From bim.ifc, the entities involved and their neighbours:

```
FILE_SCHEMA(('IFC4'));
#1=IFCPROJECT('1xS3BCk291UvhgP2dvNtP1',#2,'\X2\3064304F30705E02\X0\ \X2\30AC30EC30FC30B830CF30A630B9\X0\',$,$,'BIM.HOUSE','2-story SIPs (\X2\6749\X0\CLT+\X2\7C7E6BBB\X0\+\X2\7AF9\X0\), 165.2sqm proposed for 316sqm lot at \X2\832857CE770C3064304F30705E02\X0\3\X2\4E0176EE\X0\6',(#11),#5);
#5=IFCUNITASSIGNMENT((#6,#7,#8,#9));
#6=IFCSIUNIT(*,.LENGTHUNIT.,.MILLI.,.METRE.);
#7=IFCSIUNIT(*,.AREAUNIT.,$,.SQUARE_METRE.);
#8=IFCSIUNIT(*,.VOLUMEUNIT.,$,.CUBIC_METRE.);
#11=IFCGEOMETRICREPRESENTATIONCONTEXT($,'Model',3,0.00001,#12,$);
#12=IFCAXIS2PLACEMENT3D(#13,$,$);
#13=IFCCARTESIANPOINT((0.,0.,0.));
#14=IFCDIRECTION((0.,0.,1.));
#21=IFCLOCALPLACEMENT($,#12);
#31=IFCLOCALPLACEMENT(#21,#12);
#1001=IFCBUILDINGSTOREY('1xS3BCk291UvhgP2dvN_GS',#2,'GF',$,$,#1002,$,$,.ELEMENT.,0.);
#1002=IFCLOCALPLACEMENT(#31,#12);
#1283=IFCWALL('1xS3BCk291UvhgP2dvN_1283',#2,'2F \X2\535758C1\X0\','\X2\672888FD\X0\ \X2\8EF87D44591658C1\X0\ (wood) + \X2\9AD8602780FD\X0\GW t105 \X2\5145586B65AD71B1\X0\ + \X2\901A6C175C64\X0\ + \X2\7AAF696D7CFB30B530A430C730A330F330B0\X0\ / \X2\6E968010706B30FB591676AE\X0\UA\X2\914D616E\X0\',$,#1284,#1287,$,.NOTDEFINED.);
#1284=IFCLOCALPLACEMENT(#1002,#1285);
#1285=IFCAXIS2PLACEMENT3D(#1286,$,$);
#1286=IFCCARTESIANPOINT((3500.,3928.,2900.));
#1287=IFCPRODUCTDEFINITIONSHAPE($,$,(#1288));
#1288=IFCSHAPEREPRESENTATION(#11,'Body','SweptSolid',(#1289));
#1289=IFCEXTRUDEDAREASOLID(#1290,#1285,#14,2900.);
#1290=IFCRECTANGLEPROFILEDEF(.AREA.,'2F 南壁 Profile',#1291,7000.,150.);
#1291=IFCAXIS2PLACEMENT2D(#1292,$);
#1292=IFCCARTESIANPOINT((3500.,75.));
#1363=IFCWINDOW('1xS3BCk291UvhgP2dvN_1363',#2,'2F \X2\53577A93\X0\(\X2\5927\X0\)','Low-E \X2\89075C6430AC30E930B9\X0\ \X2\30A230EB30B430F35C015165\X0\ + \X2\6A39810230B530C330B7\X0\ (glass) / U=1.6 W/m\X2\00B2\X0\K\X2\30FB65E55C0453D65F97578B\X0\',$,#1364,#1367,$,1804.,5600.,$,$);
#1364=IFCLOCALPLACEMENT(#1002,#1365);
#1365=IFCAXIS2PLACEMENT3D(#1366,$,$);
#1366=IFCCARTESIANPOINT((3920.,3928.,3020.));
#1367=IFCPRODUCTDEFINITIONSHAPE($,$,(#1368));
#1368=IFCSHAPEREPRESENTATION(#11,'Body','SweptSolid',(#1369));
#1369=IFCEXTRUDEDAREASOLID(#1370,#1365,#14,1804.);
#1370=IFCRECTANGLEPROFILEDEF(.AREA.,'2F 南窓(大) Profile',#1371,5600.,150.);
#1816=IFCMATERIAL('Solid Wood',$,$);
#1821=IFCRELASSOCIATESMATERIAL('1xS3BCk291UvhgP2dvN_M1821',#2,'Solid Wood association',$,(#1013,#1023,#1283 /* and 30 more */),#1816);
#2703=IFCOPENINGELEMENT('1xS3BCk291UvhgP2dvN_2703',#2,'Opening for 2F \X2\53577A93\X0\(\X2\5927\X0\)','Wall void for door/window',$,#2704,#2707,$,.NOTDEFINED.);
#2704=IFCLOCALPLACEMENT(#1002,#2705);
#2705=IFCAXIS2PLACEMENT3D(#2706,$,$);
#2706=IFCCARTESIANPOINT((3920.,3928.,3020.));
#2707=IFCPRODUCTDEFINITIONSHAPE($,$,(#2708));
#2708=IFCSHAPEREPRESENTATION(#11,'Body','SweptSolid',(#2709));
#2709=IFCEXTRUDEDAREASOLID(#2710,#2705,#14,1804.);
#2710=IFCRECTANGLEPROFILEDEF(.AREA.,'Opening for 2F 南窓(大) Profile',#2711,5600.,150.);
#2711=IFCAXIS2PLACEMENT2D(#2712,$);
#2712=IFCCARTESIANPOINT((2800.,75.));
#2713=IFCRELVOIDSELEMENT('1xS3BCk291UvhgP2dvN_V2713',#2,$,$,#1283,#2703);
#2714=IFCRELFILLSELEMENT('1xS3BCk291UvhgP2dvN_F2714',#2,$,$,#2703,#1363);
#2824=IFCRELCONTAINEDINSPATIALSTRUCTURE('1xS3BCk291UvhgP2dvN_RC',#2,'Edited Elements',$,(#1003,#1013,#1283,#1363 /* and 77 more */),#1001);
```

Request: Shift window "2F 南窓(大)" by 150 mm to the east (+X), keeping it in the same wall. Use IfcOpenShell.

```python
import ifcopenshell
import ifcopenshell.api.geometry
import ifcopenshell.util.placement
import ifcopenshell.util.unit

model = ifcopenshell.open("bim.ifc")
unit_scale = ifcopenshell.util.unit.calculate_unit_scale(model)

window = model.by_guid("1xS3BCk291UvhgP2dvN_1363")
opening = window.FillsVoids[0].RelatingOpeningElement
wall = opening.VoidsElements[0].RelatingBuildingElement

wall_matrix = ifcopenshell.util.placement.get_local_placement(wall.ObjectPlacement)
shift = wall_matrix[:3, 0] * 0.15 / unit_scale
before = ifcopenshell.util.placement.get_local_placement(window.ObjectPlacement)[:3, 3].copy()

# The window is not placed relative to its opening, so move both.
for product in (opening, window):
    matrix = ifcopenshell.util.placement.get_local_placement(product.ObjectPlacement)
    matrix[:3, 3] += shift
    ifcopenshell.api.geometry.edit_object_placement(model, product=product, matrix=matrix, is_si=False)

after = ifcopenshell.util.placement.get_local_placement(window.ObjectPlacement)[:3, 3]
print("window moved by", (after - before).round(3) + 0.0)

model.write("bim_v2.ifc")
```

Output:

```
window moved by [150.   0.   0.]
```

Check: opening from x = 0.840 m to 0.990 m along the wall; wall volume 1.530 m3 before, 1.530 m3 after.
